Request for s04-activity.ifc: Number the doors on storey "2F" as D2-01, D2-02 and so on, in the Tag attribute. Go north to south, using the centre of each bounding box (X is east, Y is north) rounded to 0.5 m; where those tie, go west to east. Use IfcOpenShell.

First a look at what the model holds.

```python
import ifcopenshell
import ifcopenshell.util.element
import ifcopenshell.util.placement

model = ifcopenshell.open("s04-activity.ifc")
print(model.schema)
storey = next(s for s in model.by_type("IfcBuildingStorey") if s.Name == "2F")
doors = [e for e in ifcopenshell.util.element.get_decomposition(storey) if e.is_a("IfcDoor")]
for e in sorted(doors, key=lambda e: e.id()):
    origin = ifcopenshell.util.placement.get_local_placement(e.ObjectPlacement)[:3, 3]
    print(e.id(), e.Tag, e.Name, origin.round(2) + 0.0, sep=" | ")
```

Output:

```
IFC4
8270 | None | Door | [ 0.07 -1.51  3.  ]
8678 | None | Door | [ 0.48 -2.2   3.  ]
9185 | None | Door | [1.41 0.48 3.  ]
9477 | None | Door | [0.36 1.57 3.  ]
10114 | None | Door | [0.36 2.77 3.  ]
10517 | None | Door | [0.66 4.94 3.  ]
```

```python
import ifcopenshell
import ifcopenshell.geom
import ifcopenshell.util.element
import ifcopenshell.util.shape

model = ifcopenshell.open("s04-activity.ifc")
settings = ifcopenshell.geom.settings()
settings.set("use-world-coords", True)


def centre(element):
    shape = ifcopenshell.geom.create_shape(settings, element)
    return ifcopenshell.util.shape.get_bbox_centroid(shape.geometry)


storey = next(s for s in model.by_type("IfcBuildingStorey") if s.Name == "2F")
doors = [e for e in ifcopenshell.util.element.get_decomposition(storey) if e.is_a("IfcDoor")]

# Insertion points can sit at a corner or the storey origin, so sort by the geometry (in metres).
centres = {e: centre(e) for e in doors}
doors.sort(key=lambda e: (-round(centres[e][1] / 0.5), centres[e][0]))

for i, e in enumerate(doors, start=1):
    number = f"D2-{i:02d}"
    e.Tag = number
    print(e.id(), number)

model.write("s04-activity_edited.ifc")
```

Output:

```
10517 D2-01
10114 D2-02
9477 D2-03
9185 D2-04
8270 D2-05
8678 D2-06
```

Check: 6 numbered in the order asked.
